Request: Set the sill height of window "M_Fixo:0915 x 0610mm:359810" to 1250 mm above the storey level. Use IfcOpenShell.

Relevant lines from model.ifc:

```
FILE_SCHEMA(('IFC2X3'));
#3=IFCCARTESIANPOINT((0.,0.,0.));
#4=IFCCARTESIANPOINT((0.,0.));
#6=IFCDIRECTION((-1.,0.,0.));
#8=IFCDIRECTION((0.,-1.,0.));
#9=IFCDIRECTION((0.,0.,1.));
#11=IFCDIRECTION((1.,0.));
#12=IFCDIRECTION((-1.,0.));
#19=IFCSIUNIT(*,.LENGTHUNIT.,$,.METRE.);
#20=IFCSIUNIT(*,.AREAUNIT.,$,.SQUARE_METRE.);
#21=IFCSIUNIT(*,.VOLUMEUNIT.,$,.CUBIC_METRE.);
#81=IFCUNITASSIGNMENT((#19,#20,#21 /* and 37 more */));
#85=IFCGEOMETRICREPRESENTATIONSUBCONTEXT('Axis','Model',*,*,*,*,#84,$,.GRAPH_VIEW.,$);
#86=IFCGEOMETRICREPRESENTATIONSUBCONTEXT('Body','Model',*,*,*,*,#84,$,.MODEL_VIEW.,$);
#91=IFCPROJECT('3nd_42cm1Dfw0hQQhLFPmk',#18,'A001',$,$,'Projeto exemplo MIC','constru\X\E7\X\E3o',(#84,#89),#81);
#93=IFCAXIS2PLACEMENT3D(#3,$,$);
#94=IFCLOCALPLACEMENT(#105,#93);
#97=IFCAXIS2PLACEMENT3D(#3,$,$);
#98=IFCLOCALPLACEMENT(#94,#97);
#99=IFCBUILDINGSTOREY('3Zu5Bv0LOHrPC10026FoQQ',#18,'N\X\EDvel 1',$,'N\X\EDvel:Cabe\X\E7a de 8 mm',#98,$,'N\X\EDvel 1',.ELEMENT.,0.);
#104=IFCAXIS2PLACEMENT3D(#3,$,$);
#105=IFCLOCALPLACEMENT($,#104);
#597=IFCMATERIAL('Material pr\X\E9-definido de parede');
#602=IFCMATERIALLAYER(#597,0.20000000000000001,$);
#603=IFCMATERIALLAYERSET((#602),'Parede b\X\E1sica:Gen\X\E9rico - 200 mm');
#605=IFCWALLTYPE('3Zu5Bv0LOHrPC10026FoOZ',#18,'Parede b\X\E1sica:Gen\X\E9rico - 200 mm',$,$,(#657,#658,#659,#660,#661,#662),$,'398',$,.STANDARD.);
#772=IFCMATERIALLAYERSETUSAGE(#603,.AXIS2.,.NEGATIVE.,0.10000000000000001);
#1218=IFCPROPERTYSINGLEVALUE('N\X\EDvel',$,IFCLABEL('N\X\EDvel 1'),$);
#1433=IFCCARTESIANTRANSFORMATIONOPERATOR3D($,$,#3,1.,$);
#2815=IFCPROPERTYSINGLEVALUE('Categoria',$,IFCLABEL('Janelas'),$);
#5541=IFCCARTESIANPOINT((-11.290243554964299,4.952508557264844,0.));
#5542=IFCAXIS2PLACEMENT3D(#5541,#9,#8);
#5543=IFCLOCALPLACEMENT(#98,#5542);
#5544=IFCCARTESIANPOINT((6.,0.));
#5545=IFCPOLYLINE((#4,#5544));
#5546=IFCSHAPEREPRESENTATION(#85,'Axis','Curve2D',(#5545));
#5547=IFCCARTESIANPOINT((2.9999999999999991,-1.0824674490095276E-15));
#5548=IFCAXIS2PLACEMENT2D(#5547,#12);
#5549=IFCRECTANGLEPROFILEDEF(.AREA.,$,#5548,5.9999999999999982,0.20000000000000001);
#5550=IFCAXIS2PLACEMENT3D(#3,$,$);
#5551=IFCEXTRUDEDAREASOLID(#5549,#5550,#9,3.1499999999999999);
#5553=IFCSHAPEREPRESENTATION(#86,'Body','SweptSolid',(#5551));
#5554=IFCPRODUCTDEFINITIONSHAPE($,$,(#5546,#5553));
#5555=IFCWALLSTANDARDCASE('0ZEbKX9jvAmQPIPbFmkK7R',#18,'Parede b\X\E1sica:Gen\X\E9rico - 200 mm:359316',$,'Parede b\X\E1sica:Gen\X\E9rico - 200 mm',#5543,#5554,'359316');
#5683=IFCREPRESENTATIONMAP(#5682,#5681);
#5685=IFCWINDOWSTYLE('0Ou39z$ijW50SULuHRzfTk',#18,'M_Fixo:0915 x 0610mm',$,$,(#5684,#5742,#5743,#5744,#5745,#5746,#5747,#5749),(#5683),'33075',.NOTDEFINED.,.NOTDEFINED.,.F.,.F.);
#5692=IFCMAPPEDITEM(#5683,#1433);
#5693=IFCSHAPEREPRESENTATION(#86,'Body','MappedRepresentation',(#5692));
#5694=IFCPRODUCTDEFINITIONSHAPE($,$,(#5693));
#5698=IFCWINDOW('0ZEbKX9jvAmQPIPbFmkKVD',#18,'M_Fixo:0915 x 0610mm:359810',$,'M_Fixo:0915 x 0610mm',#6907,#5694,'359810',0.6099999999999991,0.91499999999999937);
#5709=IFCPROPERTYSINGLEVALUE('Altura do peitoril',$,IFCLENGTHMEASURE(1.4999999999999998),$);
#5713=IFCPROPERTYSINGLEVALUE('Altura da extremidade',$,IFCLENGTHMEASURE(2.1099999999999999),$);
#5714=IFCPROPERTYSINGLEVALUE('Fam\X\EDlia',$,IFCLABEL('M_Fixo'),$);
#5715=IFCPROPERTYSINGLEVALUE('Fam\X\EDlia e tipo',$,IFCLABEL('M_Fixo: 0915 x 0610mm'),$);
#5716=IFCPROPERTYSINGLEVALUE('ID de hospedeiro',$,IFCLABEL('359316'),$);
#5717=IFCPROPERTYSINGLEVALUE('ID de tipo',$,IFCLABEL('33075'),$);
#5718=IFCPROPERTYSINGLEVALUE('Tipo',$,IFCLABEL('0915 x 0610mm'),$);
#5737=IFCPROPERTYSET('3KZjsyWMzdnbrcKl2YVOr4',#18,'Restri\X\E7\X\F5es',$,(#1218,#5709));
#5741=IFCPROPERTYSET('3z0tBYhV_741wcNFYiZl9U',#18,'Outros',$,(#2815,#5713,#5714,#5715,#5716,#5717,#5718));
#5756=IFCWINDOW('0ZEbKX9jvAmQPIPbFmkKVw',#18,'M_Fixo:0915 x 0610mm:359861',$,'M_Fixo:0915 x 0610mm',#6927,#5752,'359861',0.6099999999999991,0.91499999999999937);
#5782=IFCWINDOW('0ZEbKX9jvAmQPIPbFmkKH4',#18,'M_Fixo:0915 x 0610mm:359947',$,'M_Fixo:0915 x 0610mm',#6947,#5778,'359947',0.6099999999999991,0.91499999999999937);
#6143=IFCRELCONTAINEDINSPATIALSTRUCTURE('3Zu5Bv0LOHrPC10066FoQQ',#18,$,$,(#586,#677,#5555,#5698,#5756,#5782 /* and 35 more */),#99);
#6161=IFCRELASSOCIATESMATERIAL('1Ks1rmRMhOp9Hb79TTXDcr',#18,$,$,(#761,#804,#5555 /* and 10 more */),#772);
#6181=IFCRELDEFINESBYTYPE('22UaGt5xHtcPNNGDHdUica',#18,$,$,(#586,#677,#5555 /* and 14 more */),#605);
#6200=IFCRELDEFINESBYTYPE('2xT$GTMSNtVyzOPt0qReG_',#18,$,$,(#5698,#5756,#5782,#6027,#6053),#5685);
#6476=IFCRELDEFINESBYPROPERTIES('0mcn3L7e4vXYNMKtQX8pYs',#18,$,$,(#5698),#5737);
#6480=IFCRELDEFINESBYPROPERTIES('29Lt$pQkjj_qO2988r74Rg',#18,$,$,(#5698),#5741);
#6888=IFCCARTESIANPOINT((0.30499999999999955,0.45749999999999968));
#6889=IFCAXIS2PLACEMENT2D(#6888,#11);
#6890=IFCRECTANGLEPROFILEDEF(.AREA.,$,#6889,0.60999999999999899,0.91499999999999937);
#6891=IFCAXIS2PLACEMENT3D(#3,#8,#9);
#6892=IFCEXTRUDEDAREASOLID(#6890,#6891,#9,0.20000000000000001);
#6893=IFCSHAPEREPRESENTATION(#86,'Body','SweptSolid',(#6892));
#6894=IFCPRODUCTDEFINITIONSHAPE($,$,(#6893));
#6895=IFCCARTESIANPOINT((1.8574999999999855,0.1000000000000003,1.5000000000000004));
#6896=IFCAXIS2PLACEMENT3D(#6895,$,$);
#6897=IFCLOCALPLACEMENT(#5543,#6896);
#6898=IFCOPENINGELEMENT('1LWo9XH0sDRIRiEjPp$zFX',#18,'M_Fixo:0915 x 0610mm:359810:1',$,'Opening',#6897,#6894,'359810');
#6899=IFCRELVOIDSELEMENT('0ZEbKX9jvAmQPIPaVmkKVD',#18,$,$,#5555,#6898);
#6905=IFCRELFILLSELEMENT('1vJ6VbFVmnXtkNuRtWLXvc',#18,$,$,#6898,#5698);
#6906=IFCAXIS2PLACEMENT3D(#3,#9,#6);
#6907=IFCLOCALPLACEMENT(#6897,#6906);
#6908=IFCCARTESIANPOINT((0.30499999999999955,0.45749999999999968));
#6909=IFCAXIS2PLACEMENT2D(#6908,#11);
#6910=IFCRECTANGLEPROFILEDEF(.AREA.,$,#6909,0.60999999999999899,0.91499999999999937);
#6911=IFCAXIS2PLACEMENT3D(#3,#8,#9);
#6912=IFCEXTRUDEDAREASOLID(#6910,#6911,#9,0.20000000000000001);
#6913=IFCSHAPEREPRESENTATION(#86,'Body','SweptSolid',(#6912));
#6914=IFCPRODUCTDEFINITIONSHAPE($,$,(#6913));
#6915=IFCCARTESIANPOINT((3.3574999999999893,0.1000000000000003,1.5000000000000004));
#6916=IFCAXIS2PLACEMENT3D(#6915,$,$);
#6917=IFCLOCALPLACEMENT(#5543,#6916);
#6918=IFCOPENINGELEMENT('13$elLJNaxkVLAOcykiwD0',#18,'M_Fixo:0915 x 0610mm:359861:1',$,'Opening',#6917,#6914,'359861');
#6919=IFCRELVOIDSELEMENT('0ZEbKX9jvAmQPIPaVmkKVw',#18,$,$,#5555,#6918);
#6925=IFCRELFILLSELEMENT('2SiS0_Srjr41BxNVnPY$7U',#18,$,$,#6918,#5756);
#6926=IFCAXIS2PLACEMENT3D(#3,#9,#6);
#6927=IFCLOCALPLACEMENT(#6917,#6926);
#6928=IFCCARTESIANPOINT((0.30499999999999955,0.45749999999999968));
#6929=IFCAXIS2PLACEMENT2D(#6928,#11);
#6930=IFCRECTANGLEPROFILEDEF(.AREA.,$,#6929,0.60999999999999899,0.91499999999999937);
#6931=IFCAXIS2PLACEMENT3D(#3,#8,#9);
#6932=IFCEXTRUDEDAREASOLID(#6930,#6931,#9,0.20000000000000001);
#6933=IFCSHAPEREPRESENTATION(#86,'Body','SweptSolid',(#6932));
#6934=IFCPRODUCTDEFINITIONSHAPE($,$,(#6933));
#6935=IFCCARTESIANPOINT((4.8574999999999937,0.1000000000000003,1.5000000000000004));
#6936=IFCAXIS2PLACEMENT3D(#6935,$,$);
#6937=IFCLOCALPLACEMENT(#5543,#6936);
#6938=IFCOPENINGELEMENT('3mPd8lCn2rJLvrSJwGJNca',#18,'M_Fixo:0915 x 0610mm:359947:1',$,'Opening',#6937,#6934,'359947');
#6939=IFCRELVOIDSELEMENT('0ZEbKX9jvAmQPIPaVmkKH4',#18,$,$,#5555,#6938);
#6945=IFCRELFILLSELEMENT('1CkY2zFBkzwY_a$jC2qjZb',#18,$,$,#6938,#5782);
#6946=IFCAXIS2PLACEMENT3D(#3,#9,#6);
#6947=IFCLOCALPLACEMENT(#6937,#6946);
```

```python
import numpy as np
import ifcopenshell
import ifcopenshell.api.geometry
import ifcopenshell.api.pset
import ifcopenshell.geom
import ifcopenshell.util.element
import ifcopenshell.util.placement
import ifcopenshell.util.shape
import ifcopenshell.util.unit

model = ifcopenshell.open("model.ifc")
unit_scale = ifcopenshell.util.unit.calculate_unit_scale(model)

window = model.by_guid("0ZEbKX9jvAmQPIPbFmkKVD")
opening = window.FillsVoids[0].RelatingOpeningElement
storey = ifcopenshell.util.element.get_container(window, ifc_class="IfcBuildingStorey")
level = ifcopenshell.util.placement.get_local_placement(storey.ObjectPlacement)[2, 3]

# The opening's origin need not be at the sill, so measure its lowest point.
shape = ifcopenshell.geom.create_shape(ifcopenshell.geom.settings(), opening)
bottom = ifcopenshell.util.shape.get_shape_bottom_elevation(shape, shape.geometry) / unit_scale
dz = level + 1.25 / unit_scale - bottom

shift = np.array([0.0, 0.0, dz])
# The window is placed relative to its opening, so it follows when the opening moves.
matrix = ifcopenshell.util.placement.get_local_placement(opening.ObjectPlacement)
matrix[:3, 3] += shift
ifcopenshell.api.geometry.edit_object_placement(
    model, product=opening, matrix=matrix, is_si=False, should_transform_children=True
)

# Keep the stored heights in step.
pset = model.by_id(ifcopenshell.util.element.get_pset(window, "Restrições", should_inherit=False)["id"])
ifcopenshell.api.pset.edit_pset(model, pset=pset, properties={
    "Altura do peitoril": model.create_entity("IfcLengthMeasure", ifcopenshell.util.element.get_pset(window, "Restrições", "Altura do peitoril") + dz),
})
pset = model.by_id(ifcopenshell.util.element.get_pset(window, "Outros", should_inherit=False)["id"])
ifcopenshell.api.pset.edit_pset(model, pset=pset, properties={
    "Altura da extremidade": model.create_entity("IfcLengthMeasure", ifcopenshell.util.element.get_pset(window, "Outros", "Altura da extremidade") + dz),
})

print(f"moved by {dz * unit_scale:+.3f} m")

model.write("model-out.ifc")
```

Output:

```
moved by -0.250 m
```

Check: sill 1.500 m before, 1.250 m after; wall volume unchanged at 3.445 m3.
